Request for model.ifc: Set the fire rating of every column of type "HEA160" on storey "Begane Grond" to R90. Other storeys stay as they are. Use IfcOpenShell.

First a look at what the model holds.

```python
import ifcopenshell
import ifcopenshell.util.element

model = ifcopenshell.open("model.ifc")
print(model.schema)
storey = next(s for s in model.by_type("IfcBuildingStorey") if s.Name == "Begane Grond")
columns = [e for e in ifcopenshell.util.element.get_decomposition(storey) if e.is_a("IfcColumn")]
seen = {}
for e in columns:
    element_type = ifcopenshell.util.element.get_type(e)
    key = (element_type.Name if element_type != e and element_type else None, ifcopenshell.util.element.get_pset(e, "Pset_ColumnCommon", "FireRating"))
    seen[key] = seen.get(key, 0) + 1
for (name, value), count in sorted(seen.items(), key=str):
    print(count, "x", name, "|", value)
```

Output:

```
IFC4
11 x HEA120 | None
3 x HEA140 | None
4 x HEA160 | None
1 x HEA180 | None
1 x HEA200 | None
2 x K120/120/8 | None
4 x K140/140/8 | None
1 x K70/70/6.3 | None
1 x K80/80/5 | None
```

```python
import ifcopenshell
import ifcopenshell.api.pset
import ifcopenshell.util.element

model = ifcopenshell.open("model.ifc")

storey = next(s for s in model.by_type("IfcBuildingStorey") if s.Name == "Begane Grond")
columns = [e for e in ifcopenshell.util.element.get_decomposition(storey) if e.is_a("IfcColumn")]

count = 0
for e in columns:
    element_type = ifcopenshell.util.element.get_type(e)
    if element_type in (None, e) or element_type.Name != "HEA160":
        continue
    # add_pset returns the element's existing set when there is one.
    pset = ifcopenshell.api.pset.add_pset(model, product=e, name="Pset_ColumnCommon")
    ifcopenshell.api.pset.edit_pset(model, pset=pset, properties={"FireRating": "R90"})
    count += 1

print(count, "columns updated")

model.write("model_updated.ifc")
```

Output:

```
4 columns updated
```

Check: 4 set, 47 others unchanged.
